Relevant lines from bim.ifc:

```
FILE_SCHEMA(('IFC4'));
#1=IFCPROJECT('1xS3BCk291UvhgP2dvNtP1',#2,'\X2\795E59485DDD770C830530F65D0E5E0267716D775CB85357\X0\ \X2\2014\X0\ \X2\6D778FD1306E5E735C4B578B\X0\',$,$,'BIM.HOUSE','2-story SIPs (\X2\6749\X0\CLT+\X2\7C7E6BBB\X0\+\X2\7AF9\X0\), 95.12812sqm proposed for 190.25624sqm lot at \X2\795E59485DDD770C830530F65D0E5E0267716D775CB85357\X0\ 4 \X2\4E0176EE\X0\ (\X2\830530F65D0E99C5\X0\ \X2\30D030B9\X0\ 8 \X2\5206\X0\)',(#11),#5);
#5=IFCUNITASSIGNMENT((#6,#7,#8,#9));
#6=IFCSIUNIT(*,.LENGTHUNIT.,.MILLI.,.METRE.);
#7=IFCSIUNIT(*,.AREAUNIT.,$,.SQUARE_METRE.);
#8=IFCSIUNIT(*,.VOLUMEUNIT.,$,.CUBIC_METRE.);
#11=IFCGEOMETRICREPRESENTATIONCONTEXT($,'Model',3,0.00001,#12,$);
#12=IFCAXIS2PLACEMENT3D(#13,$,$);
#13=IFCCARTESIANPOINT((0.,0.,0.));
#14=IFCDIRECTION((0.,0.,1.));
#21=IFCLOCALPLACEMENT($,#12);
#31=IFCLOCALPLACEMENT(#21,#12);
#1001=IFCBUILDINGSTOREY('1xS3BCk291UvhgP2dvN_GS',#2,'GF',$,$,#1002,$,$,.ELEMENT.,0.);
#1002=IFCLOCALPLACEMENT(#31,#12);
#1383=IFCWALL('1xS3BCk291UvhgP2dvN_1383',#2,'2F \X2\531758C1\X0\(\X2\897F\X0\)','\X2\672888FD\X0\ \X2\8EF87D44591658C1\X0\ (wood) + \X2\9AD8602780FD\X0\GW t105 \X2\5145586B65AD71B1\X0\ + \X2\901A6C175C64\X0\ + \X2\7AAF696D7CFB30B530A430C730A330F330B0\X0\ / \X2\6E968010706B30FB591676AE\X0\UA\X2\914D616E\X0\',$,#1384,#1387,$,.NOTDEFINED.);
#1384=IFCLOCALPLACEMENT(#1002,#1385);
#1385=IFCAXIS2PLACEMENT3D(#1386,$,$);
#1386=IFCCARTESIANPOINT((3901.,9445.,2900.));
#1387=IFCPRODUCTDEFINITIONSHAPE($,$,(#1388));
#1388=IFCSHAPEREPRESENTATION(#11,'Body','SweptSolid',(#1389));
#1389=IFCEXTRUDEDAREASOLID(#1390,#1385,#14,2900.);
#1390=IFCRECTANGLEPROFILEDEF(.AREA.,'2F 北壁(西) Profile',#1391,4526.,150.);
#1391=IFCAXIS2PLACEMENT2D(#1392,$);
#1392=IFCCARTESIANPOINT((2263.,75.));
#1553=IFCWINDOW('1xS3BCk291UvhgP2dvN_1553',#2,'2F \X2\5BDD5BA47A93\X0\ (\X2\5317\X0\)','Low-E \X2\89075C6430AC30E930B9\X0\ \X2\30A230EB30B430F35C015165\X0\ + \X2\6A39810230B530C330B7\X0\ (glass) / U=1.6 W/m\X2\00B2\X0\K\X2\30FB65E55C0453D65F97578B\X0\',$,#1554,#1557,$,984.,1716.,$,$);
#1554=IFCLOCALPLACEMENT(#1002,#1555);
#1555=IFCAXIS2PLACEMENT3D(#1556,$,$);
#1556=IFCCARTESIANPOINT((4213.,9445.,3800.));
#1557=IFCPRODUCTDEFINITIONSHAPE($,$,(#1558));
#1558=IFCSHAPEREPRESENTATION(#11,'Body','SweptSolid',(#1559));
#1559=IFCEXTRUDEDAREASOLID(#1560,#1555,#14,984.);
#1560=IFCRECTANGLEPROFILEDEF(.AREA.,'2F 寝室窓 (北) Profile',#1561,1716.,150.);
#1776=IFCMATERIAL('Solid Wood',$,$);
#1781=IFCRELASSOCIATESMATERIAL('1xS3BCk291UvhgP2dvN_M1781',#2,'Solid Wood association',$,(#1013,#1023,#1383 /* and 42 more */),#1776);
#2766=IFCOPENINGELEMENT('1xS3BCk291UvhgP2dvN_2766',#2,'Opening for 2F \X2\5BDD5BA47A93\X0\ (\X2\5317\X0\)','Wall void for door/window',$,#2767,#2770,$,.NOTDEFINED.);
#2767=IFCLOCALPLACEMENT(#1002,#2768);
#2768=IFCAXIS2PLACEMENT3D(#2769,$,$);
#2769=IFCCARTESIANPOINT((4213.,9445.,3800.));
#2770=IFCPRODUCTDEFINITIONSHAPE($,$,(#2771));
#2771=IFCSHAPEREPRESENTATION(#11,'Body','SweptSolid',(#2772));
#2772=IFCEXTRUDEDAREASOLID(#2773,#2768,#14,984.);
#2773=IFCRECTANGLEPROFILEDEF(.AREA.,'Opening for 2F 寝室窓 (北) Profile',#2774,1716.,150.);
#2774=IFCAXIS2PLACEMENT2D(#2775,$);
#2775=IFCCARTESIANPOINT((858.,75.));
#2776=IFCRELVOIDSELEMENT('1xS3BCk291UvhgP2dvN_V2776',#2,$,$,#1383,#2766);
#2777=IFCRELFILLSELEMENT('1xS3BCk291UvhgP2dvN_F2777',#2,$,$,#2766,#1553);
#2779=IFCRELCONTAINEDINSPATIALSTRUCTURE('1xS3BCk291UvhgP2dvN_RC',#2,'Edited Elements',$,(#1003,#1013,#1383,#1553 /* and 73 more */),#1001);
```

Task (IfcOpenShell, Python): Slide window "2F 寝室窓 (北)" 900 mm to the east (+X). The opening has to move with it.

```python
import ifcopenshell
import ifcopenshell.api.geometry
import ifcopenshell.util.placement

model = ifcopenshell.open("bim.ifc")

window = model.by_guid("1xS3BCk291UvhgP2dvN_1553")
opening = window.FillsVoids[0].RelatingOpeningElement
wall = opening.VoidsElements[0].RelatingBuildingElement

wall_matrix = ifcopenshell.util.placement.get_local_placement(wall.ObjectPlacement)
shift = wall_matrix[:3, 0] * 900.0
before = ifcopenshell.util.placement.get_local_placement(window.ObjectPlacement)[:3, 3].copy()

# The window is not placed relative to its opening, so move both.
for product in (opening, window):
    matrix = ifcopenshell.util.placement.get_local_placement(product.ObjectPlacement)
    matrix[:3, 3] += shift
    ifcopenshell.api.geometry.edit_object_placement(model, product=product, matrix=matrix, is_si=False)

after = ifcopenshell.util.placement.get_local_placement(window.ObjectPlacement)[:3, 3]
print("window moved by", (after - before).round(3) + 0.0)

model.write("bim_v2.ifc")
```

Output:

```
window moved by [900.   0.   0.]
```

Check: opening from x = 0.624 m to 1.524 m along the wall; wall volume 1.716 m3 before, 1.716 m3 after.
